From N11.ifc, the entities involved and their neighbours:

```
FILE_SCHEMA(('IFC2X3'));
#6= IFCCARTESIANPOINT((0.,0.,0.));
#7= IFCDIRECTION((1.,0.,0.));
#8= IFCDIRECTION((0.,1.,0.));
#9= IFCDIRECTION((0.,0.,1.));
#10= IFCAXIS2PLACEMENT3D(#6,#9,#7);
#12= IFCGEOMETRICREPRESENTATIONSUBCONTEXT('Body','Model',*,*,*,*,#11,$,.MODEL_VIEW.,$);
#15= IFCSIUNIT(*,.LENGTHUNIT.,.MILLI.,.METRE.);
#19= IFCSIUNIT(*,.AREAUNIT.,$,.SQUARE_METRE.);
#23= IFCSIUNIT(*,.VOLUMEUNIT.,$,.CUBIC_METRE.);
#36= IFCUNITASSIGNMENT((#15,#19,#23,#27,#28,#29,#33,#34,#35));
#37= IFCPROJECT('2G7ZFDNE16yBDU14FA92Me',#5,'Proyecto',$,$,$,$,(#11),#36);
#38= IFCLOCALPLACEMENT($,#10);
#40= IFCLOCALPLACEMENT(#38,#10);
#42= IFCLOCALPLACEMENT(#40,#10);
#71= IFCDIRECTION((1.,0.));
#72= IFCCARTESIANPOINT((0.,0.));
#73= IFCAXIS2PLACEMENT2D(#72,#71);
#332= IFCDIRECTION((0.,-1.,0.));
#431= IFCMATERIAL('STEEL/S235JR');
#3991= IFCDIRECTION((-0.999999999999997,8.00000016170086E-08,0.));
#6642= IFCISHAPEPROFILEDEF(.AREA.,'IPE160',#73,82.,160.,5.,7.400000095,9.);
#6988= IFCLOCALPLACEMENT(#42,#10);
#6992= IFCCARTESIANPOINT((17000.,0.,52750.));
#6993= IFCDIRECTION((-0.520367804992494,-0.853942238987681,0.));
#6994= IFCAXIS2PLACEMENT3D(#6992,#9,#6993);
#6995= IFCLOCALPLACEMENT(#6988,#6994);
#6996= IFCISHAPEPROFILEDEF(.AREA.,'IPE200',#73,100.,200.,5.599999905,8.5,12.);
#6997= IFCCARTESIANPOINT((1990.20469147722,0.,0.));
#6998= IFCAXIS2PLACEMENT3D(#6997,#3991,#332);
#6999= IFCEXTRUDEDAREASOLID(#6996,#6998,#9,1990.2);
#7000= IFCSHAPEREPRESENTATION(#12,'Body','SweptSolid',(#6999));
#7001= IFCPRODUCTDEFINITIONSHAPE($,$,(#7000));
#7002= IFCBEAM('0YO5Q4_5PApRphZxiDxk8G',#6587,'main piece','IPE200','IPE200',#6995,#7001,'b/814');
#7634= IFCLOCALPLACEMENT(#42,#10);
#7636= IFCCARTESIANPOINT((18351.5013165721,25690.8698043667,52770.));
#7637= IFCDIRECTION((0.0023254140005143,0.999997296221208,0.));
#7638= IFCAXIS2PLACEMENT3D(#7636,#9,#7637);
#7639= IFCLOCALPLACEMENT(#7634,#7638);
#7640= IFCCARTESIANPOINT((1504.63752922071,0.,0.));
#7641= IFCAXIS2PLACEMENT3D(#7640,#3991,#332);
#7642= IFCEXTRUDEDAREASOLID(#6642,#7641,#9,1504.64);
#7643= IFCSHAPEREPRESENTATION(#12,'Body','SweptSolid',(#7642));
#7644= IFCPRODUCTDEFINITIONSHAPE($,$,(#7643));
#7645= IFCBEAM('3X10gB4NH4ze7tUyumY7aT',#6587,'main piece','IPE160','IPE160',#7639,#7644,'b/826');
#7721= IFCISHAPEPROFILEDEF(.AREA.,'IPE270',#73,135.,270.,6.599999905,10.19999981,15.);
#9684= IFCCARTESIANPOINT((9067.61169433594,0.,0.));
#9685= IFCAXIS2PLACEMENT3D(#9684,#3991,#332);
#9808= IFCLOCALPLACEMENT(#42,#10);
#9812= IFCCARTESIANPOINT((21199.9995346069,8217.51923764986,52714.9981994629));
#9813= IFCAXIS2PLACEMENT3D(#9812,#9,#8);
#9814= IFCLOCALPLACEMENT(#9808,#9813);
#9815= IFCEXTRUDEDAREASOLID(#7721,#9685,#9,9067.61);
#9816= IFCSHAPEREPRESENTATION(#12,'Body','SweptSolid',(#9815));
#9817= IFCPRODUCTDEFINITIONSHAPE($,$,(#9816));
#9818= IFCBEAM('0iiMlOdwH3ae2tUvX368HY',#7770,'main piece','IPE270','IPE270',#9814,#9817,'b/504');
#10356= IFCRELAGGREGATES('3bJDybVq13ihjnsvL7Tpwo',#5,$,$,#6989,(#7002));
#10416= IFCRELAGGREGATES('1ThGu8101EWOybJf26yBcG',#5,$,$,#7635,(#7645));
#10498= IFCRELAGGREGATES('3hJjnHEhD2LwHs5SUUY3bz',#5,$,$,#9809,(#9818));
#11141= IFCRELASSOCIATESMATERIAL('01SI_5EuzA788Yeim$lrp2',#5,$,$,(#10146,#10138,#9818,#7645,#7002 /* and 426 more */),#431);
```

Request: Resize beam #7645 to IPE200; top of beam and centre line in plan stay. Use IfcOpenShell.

```python
import ifcopenshell
import ifcopenshell.util.element
import ifcopenshell.util.representation

model = ifcopenshell.open("N11.ifc")

member = model.by_guid("3X10gB4NH4ze7tUyumY7aT")
source = next(p for p in model.by_type("IfcIShapeProfileDef") if p.ProfileName == "IPE200")

body = ifcopenshell.util.representation.get_representation(member, "Model", "Body")
solid = body.Items[0]
old_profile = solid.SweptArea

# Copy the section's sizes but keep this member's own profile position.
profile = ifcopenshell.util.element.copy(model, source)
# Profiles are centred, so shift by half the change in depth to hold the top.
shift = (old_profile.OverallDepth - profile.OverallDepth) / 2
x, y = old_profile.Position.Location.Coordinates
up = (0.0, 1.0)  # upwards, in the solid's own plane
location = model.createIfcCartesianPoint((x + up[0] * shift, y + up[1] * shift))
profile.Position = model.createIfcAxis2Placement2D(location, old_profile.Position.RefDirection)
solid.SweptArea = profile
if not model.get_total_inverses(old_profile):
    ifcopenshell.util.element.remove_deep2(model, old_profile)
member.Description = member.Description.replace("IPE160", "IPE200")
member.ObjectType = member.ObjectType.replace("IPE160", "IPE200")

print(solid.SweptArea)

model.write("N11-out.ifc")
```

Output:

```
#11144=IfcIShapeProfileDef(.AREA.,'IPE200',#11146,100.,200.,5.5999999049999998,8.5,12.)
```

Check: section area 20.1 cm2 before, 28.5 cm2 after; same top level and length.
